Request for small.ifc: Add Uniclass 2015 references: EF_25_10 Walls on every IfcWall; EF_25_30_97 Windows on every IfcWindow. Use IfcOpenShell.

First a look at what the model holds.

```python
import ifcopenshell

model = ifcopenshell.open("small.ifc")
print(model.schema)
print("classifications:", [c.Name for c in model.by_type("IfcClassification")])
for ifc_class in ("IfcDoor", "IfcRoof", "IfcStair", "IfcWall", "IfcWindow"):
    print(ifc_class, len(model.by_type(ifc_class)))
```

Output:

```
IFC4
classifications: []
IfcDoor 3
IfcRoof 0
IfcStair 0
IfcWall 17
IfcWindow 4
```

```python
import ifcopenshell
import ifcopenshell.api.classification

model = ifcopenshell.open("small.ifc")

system = ifcopenshell.api.classification.add_classification(model, classification="Uniclass 2015")

codes = {
    "IfcWall": ("EF_25_10", "Walls"),
    "IfcWindow": ("EF_25_30_97", "Windows"),
}
for ifc_class, (code, name) in codes.items():
    products = model.by_type(ifc_class)
    ifcopenshell.api.classification.add_reference(
        model, products=products, classification=system, identification=code, name=name
    )
    print(code, len(products))

model.write("small_rev.ifc")
```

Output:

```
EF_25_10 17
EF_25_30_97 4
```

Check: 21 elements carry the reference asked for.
